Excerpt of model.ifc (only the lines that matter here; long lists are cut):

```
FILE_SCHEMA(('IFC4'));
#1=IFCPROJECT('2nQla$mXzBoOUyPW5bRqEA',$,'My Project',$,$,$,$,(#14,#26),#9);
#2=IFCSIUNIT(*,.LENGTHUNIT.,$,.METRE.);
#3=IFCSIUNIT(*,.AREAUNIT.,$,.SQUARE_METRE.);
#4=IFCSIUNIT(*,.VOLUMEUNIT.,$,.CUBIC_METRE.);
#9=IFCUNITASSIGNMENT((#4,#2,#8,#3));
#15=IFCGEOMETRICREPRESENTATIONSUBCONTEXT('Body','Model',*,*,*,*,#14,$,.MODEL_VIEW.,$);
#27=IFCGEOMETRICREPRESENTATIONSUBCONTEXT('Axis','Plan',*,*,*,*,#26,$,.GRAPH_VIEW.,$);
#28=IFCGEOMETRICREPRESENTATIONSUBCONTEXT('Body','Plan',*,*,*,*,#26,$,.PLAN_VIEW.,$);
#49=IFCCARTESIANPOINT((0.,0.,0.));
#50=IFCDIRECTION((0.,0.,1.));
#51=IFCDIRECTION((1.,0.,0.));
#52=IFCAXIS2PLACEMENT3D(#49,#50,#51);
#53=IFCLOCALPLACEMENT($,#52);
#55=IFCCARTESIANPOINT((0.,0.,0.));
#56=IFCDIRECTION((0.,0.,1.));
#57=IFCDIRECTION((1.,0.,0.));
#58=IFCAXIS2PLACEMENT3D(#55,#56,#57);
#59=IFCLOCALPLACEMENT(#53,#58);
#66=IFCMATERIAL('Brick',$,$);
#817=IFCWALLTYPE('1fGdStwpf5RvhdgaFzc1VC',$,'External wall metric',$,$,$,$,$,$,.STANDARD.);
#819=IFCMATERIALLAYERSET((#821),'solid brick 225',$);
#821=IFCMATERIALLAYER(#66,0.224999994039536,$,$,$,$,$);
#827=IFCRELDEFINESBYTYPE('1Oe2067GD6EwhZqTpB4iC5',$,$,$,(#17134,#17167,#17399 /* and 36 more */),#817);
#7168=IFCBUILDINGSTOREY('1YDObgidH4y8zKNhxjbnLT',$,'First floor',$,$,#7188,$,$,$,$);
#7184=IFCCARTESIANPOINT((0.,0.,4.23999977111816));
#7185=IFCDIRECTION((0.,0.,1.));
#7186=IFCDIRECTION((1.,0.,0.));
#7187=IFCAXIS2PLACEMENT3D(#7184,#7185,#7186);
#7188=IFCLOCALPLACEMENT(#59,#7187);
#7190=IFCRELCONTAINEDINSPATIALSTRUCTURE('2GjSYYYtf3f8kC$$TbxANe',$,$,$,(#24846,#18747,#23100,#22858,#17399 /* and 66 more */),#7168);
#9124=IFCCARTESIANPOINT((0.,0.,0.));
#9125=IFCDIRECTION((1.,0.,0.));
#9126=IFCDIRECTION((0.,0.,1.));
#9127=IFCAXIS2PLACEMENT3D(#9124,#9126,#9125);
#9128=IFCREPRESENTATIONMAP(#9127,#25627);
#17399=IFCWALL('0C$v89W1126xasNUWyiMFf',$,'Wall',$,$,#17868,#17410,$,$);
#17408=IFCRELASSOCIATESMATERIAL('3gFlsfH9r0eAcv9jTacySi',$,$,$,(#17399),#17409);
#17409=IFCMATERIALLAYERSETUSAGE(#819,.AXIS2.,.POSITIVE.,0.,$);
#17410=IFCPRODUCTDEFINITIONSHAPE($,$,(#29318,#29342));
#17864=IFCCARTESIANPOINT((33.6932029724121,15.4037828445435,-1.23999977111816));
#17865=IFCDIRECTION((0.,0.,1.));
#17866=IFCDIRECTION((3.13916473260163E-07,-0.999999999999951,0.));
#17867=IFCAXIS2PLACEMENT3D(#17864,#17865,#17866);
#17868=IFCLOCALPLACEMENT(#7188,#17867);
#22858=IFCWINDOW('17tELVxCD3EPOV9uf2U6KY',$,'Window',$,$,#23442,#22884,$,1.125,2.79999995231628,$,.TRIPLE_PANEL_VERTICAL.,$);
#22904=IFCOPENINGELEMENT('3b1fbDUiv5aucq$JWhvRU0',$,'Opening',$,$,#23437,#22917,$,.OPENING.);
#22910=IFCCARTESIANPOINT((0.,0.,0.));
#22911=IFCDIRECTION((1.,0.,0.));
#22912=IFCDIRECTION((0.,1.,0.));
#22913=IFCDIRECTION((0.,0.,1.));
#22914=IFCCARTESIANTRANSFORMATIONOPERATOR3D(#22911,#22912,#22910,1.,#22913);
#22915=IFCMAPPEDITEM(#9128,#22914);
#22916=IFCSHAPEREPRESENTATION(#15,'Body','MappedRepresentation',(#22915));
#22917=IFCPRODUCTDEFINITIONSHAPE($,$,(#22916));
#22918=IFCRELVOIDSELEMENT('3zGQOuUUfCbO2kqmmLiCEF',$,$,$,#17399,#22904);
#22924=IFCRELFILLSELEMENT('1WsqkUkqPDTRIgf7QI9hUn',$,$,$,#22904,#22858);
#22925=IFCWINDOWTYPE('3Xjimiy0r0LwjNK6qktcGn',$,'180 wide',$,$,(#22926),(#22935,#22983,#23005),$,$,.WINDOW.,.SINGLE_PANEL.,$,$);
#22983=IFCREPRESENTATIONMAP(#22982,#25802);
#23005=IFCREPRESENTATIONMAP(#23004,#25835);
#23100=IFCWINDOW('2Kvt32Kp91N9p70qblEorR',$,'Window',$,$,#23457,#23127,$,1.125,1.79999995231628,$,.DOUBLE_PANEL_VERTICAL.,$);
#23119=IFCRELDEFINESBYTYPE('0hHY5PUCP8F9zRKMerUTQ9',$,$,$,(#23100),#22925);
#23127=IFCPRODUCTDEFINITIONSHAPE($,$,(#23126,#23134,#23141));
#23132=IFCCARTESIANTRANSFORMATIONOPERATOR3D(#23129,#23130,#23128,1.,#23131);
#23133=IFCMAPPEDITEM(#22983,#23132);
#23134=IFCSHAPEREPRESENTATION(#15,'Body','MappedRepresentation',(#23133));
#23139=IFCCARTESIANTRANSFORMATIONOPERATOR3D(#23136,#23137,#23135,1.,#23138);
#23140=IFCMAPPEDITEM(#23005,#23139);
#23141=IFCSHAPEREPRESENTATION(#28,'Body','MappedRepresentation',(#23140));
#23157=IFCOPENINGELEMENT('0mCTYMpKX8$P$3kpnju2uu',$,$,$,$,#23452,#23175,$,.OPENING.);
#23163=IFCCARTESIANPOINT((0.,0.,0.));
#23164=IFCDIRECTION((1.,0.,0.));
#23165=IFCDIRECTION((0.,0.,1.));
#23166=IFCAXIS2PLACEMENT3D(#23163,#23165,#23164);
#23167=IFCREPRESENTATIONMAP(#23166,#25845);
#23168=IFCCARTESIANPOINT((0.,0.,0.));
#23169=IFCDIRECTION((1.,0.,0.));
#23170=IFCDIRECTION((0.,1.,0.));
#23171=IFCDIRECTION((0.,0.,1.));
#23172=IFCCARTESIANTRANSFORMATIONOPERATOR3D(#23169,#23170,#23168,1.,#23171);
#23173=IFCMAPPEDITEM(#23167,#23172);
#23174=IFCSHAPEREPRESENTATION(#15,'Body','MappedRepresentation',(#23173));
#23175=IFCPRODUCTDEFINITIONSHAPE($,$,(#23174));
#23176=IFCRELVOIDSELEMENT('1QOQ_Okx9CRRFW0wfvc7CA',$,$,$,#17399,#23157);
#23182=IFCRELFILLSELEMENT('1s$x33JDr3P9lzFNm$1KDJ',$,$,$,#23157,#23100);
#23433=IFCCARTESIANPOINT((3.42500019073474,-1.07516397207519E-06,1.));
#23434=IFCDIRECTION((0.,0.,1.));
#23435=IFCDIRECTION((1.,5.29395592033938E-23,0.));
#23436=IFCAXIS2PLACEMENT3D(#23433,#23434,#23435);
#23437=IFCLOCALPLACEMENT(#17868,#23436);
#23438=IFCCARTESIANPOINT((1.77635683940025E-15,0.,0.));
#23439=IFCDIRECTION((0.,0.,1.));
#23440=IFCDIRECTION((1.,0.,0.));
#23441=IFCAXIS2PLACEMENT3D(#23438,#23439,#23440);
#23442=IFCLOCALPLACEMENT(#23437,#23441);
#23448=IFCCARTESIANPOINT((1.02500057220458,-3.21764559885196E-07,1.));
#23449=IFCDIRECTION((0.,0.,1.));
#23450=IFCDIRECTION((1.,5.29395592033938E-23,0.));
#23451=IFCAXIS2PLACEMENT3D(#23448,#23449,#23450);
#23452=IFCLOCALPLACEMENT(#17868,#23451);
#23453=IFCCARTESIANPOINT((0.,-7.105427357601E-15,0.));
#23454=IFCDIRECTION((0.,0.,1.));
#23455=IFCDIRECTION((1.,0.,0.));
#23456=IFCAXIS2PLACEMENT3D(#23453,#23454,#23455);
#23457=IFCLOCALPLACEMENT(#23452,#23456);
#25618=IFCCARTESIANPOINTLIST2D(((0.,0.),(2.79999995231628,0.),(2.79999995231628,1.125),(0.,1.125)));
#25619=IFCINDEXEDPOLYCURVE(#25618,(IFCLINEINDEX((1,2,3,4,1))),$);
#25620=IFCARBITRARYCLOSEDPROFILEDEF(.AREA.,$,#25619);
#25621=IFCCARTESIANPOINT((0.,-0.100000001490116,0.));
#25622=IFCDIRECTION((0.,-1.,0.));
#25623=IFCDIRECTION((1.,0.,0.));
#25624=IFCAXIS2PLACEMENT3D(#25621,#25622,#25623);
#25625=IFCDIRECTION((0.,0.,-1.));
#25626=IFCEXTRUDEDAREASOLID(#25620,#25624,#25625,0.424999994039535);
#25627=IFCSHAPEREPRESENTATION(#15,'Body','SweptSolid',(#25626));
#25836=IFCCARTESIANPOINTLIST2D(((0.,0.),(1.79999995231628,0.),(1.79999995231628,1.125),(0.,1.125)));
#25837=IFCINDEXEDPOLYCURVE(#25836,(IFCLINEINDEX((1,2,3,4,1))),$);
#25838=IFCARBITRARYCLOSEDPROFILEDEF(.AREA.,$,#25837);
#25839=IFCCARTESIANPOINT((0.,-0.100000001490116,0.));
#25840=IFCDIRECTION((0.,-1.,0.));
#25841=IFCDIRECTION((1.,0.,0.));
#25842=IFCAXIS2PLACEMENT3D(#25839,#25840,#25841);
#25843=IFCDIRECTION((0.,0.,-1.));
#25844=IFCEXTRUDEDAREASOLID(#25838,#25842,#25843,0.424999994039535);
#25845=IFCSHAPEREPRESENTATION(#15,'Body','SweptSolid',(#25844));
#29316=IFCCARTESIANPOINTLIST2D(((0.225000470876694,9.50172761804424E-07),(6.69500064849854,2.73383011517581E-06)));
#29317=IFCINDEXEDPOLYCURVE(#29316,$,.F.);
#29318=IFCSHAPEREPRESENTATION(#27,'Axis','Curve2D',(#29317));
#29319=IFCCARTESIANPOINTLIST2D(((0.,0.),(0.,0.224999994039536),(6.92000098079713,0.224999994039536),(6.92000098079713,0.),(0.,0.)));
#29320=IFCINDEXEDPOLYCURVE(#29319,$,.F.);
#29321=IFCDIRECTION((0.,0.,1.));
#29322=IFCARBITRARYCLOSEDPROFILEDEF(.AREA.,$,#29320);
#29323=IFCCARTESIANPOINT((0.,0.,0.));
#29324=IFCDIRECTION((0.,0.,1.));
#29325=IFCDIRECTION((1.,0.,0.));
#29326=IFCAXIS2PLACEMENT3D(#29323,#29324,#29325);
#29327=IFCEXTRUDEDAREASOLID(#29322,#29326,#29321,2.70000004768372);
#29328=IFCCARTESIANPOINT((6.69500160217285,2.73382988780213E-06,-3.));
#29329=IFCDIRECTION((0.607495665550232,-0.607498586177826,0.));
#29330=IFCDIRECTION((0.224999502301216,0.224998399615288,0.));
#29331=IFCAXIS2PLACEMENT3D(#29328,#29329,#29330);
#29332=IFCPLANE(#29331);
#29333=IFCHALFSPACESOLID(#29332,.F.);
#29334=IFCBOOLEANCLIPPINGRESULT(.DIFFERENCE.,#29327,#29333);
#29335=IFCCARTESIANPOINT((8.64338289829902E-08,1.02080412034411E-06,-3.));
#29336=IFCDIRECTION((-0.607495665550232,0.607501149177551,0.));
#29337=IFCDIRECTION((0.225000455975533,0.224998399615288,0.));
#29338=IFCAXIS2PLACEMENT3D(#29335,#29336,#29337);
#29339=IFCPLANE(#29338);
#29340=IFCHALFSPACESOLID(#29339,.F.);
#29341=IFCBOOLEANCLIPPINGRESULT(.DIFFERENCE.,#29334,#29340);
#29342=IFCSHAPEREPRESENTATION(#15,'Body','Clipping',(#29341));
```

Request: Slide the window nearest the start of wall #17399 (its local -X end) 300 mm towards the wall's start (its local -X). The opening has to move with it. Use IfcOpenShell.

```python
import ifcopenshell
import ifcopenshell.api.geometry
import ifcopenshell.util.placement

model = ifcopenshell.open("model.ifc")

window = model.by_id(23100)
opening = window.FillsVoids[0].RelatingOpeningElement
wall = opening.VoidsElements[0].RelatingBuildingElement

wall_matrix = ifcopenshell.util.placement.get_local_placement(wall.ObjectPlacement)
shift = wall_matrix[:3, 0] * -0.3
before = ifcopenshell.util.placement.get_local_placement(window.ObjectPlacement)[:3, 3].copy()

# The window is placed relative to its opening, so it follows when the opening moves.
matrix = ifcopenshell.util.placement.get_local_placement(opening.ObjectPlacement)
matrix[:3, 3] += shift
ifcopenshell.api.geometry.edit_object_placement(
    model, product=opening, matrix=matrix, is_si=False, should_transform_children=True
)

after = ifcopenshell.util.placement.get_local_placement(window.ObjectPlacement)[:3, 3]
print("window moved by", (after - before).round(3) + 0.0)

model.write("model_edited.ifc")
```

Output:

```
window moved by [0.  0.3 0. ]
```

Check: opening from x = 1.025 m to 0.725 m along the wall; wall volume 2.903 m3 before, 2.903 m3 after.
